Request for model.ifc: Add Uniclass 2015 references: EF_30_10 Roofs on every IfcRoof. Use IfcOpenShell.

First a look at what the model holds.

```python
import ifcopenshell

model = ifcopenshell.open("model.ifc")
print(model.schema)
print("classifications:", [c.Name for c in model.by_type("IfcClassification")])
for ifc_class in ("IfcDoor", "IfcRoof", "IfcStair", "IfcWall", "IfcWindow"):
    print(ifc_class, len(model.by_type(ifc_class)))
```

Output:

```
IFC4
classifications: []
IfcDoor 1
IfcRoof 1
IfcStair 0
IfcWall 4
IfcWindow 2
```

```python
import ifcopenshell
import ifcopenshell.api.classification

model = ifcopenshell.open("model.ifc")

system = ifcopenshell.api.classification.add_classification(model, classification="Uniclass 2015")

codes = {
    "IfcRoof": ("EF_30_10", "Roofs"),
}
for ifc_class, (code, name) in codes.items():
    products = model.by_type(ifc_class)
    ifcopenshell.api.classification.add_reference(
        model, products=products, classification=system, identification=code, name=name
    )
    print(code, len(products))

model.write("model_edited.ifc")
```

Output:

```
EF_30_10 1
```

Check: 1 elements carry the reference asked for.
